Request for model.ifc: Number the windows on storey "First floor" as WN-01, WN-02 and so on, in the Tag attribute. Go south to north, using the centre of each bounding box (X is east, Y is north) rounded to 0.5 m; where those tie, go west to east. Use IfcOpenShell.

First a look at what the model holds.

```python
import ifcopenshell
import ifcopenshell.util.element
import ifcopenshell.util.placement

model = ifcopenshell.open("model.ifc")
print(model.schema)
storey = next(s for s in model.by_type("IfcBuildingStorey") if s.Name == "First floor")
windows = [e for e in ifcopenshell.util.element.get_decomposition(storey) if e.is_a("IfcWindow")]
for e in sorted(windows, key=lambda e: e.id()):
    origin = ifcopenshell.util.placement.get_local_placement(e.ObjectPlacement)[:3, 3]
    print(e.id(), e.Tag, e.Name, origin.round(2) + 0.0, sep=" | ")
```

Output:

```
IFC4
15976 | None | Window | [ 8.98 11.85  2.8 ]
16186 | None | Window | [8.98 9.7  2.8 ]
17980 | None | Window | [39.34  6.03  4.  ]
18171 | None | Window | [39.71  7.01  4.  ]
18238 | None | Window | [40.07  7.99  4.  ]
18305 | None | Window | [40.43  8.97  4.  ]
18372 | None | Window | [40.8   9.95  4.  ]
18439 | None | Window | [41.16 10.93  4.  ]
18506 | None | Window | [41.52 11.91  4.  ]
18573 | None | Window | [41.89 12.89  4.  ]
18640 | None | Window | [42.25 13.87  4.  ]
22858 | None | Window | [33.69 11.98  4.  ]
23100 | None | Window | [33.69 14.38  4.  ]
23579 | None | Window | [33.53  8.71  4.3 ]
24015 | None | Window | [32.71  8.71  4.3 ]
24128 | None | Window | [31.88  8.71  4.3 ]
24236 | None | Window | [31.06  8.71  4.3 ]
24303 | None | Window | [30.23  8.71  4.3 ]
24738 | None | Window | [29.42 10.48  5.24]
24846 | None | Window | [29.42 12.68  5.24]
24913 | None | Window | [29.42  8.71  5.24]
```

```python
import ifcopenshell
import ifcopenshell.geom
import ifcopenshell.util.element
import ifcopenshell.util.shape

model = ifcopenshell.open("model.ifc")
settings = ifcopenshell.geom.settings()
settings.set("use-world-coords", True)


def centre(element):
    shape = ifcopenshell.geom.create_shape(settings, element)
    return ifcopenshell.util.shape.get_bbox_centroid(shape.geometry)


storey = next(s for s in model.by_type("IfcBuildingStorey") if s.Name == "First floor")
windows = [e for e in ifcopenshell.util.element.get_decomposition(storey) if e.is_a("IfcWindow")]

# Insertion points can sit at a corner or the storey origin, so sort by the geometry (in metres).
centres = {e: centre(e) for e in windows}
windows.sort(key=lambda e: (round(centres[e][1] / 0.5), centres[e][0]))

for i, e in enumerate(windows, start=1):
    number = f"WN-{i:02d}"
    e.Tag = number
    print(e.id(), number)

model.write("model-out.ifc")
```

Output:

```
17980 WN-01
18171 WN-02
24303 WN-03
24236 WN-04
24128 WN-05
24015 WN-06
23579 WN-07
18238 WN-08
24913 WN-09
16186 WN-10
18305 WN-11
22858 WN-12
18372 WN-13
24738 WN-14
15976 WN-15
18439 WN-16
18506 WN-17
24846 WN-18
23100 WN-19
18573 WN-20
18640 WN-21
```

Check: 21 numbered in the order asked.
